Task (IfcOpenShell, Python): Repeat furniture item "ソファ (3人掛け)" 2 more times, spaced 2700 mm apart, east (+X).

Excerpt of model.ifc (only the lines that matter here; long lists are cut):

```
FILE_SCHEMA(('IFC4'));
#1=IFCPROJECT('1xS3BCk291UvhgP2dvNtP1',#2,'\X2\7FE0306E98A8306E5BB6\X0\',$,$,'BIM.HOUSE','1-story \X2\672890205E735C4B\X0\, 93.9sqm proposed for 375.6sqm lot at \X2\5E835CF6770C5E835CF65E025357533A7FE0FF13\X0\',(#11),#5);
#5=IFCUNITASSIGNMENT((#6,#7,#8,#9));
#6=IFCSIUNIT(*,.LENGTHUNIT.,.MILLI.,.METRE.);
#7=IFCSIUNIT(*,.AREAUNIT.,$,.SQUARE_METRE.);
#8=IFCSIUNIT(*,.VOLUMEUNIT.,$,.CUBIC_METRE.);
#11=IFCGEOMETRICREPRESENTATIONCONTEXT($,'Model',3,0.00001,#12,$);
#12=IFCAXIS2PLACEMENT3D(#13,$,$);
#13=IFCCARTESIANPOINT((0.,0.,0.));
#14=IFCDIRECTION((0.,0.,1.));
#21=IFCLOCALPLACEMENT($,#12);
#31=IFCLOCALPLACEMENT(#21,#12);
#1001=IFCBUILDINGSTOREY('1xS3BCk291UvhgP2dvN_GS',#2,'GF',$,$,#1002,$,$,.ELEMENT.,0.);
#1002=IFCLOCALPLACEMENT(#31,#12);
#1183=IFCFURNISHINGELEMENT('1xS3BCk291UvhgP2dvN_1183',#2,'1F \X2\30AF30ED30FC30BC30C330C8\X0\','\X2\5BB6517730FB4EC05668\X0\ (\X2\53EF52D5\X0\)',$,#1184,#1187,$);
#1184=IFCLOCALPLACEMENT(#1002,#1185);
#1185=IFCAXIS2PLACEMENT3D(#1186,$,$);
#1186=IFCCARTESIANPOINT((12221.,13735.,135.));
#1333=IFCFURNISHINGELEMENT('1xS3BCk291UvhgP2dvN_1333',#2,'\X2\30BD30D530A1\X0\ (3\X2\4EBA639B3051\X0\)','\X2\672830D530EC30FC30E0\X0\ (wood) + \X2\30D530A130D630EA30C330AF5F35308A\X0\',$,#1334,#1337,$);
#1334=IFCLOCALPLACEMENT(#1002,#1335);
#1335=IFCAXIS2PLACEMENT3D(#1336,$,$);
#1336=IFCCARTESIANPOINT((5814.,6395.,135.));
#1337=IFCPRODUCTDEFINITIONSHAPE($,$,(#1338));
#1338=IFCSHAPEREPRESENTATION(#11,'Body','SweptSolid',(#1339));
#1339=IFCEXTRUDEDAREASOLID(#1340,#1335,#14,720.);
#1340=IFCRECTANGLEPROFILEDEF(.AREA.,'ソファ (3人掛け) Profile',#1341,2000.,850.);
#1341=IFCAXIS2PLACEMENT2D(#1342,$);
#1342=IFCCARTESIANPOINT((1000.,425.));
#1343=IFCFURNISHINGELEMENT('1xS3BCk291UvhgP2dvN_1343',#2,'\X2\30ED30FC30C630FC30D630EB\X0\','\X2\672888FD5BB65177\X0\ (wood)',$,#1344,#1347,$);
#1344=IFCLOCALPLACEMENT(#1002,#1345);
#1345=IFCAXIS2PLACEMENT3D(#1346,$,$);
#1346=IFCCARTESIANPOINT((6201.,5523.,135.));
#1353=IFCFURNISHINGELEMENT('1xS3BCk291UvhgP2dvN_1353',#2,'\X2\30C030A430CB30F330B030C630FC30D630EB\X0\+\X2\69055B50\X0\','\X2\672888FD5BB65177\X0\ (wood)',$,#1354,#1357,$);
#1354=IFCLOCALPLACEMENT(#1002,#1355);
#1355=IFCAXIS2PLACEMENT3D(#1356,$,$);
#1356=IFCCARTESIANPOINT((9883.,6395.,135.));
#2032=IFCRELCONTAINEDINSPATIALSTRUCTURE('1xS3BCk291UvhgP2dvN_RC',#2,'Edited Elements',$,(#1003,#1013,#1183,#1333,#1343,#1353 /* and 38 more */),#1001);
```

```python
import numpy as np
import ifcopenshell
import ifcopenshell.api.geometry
import ifcopenshell.api.root
import ifcopenshell.util.element
import ifcopenshell.util.placement

model = ifcopenshell.open("model.ifc")


def reuse_history(source, copy):
    """copy_class also copies each property set's owner history, people and application; keep the originals."""
    for rel in copy.IsDefinedBy:
        if rel.is_a("IfcRelDefinesByProperties") and (history := rel.RelatingPropertyDefinition.OwnerHistory):
            rel.RelatingPropertyDefinition.OwnerHistory = source.OwnerHistory
            ifcopenshell.util.element.remove_deep2(model, history)


source = model.by_guid("1xS3BCk291UvhgP2dvN_1333")
base = ifcopenshell.util.placement.get_local_placement(source.ObjectPlacement)
step = np.array([1.0, 0.0, 0.0]) * 2700.0

for i in range(1, 3):
    copy = ifcopenshell.api.root.copy_class(model, product=source)
    copy.Representation = ifcopenshell.util.element.copy_deep(
        model, source.Representation, exclude=["IfcGeometricRepresentationContext", "IfcRepresentationMap"]
    )
    reuse_history(source, copy)
    matrix = base.copy()
    matrix[:3, 3] += i * step
    print("added at", matrix[:3, 3].round(3) + 0.0)
    ifcopenshell.api.geometry.edit_object_placement(model, product=copy, matrix=matrix, is_si=False)

model.write("model_updated.ifc")
```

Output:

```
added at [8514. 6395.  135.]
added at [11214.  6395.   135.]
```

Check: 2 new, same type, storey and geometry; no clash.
